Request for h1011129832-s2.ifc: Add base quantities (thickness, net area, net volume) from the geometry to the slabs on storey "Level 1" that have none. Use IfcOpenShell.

First a look at what the model holds.

```python
import ifcopenshell
import ifcopenshell.util.element
import ifcopenshell.util.unit

model = ifcopenshell.open("h1011129832-s2.ifc")
print(model.schema)
for unit_type in ("LENGTHUNIT", "AREAUNIT", "VOLUMEUNIT"):
    print(unit_type, ifcopenshell.util.unit.calculate_unit_scale(model, unit_type))
storey = next(s for s in model.by_type("IfcBuildingStorey") if s.Name == "Level 1")
slabs = [e for e in ifcopenshell.util.element.get_decomposition(storey) if e.is_a("IfcSlab")]
for e in sorted(slabs, key=lambda e: e.id()):
    print(e.id(), e.is_a(), e.Name, list(ifcopenshell.util.element.get_psets(e, qtos_only=True)), sep=" | ")
```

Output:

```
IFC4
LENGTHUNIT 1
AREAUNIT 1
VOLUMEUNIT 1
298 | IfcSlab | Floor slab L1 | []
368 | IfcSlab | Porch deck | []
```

```python
import ifcopenshell
import ifcopenshell.api.pset
import ifcopenshell.geom
import ifcopenshell.util.element
import ifcopenshell.util.shape
import ifcopenshell.util.unit

model = ifcopenshell.open("h1011129832-s2.ifc")
unit_scale = ifcopenshell.util.unit.calculate_unit_scale(model)
area_scale = ifcopenshell.util.unit.calculate_unit_scale(model, "AREAUNIT")
volume_scale = ifcopenshell.util.unit.calculate_unit_scale(model, "VOLUMEUNIT")
settings = ifcopenshell.geom.settings()

storey = next(s for s in model.by_type("IfcBuildingStorey") if s.Name == "Level 1")
slabs = [e for e in ifcopenshell.util.element.get_decomposition(storey) if e.is_a("IfcSlab")]

for e in sorted(slabs, key=lambda e: e.id()):
    if ifcopenshell.util.element.get_psets(e, qtos_only=True, should_inherit=False):
        continue
    # Geometry comes back in metres, in the element's own axes.
    shape = ifcopenshell.geom.create_shape(settings, e)
    values = {
        "Width": ifcopenshell.util.shape.get_z(shape.geometry) / unit_scale,
        "NetArea": ifcopenshell.util.shape.get_footprint_area(shape.geometry) / area_scale,
        "NetVolume": ifcopenshell.util.shape.get_volume(shape.geometry) / volume_scale,
    }
    qto = ifcopenshell.api.pset.add_qto(model, product=e, name="Qto_SlabBaseQuantities")
    ifcopenshell.api.pset.edit_qto(model, qto=qto, properties=values)
    print(e.id(), {k: round(v, 3) for k, v in values.items()})

model.write("h1011129832-s2_edited.ifc")
```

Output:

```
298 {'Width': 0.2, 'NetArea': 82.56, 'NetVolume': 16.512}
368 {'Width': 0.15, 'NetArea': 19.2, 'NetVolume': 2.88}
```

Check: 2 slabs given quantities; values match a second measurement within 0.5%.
